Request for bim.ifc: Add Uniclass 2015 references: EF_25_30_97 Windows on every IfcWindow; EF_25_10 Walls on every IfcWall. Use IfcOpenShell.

First a look at what the model holds.

```python
import ifcopenshell

model = ifcopenshell.open("bim.ifc")
print(model.schema)
print("classifications:", [c.Name for c in model.by_type("IfcClassification")])
for ifc_class in ("IfcDoor", "IfcRoof", "IfcStair", "IfcWall", "IfcWindow"):
    print(ifc_class, len(model.by_type(ifc_class)))
```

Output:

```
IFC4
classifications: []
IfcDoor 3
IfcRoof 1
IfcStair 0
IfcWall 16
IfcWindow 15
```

```python
import ifcopenshell
import ifcopenshell.api.classification

model = ifcopenshell.open("bim.ifc")

system = ifcopenshell.api.classification.add_classification(model, classification="Uniclass 2015")

codes = {
    "IfcWindow": ("EF_25_30_97", "Windows"),
    "IfcWall": ("EF_25_10", "Walls"),
}
for ifc_class, (code, name) in codes.items():
    products = model.by_type(ifc_class)
    ifcopenshell.api.classification.add_reference(
        model, products=products, classification=system, identification=code, name=name
    )
    print(code, len(products))

model.write("bim_edited.ifc")
```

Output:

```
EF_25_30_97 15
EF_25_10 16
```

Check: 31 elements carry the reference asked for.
